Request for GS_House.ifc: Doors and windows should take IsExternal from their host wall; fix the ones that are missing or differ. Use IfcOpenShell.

First a look at what the model holds.

```python
import ifcopenshell
import ifcopenshell.util.element

model = ifcopenshell.open("GS_House.ifc")
print(model.schema)
seen = {}
for e in model.by_type("IfcDoor") + model.by_type("IfcWindow"):
    if not e.FillsVoids:
        continue
    host = e.FillsVoids[0].RelatingOpeningElement.VoidsElements[0].RelatingBuildingElement
    own = ifcopenshell.util.element.get_pset(e, f"Pset_{e.is_a()[3:].removesuffix('StandardCase')}Common", "IsExternal")
    wall = ifcopenshell.util.element.get_pset(host, "Pset_WallCommon", "IsExternal")
    seen[e.is_a(), own, wall] = seen.get((e.is_a(), own, wall), 0) + 1
for (cls, own, wall), count in sorted(seen.items(), key=str):
    print(count, cls, "IsExternal:", own, "| host wall:", wall)
```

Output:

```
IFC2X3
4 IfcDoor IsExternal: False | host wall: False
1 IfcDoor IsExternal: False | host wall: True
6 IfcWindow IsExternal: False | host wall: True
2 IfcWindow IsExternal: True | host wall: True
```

```python
import ifcopenshell
import ifcopenshell.api.pset
import ifcopenshell.util.element

model = ifcopenshell.open("GS_House.ifc")

count = 0
for ifc_class, pset_name in (("IfcDoor", "Pset_DoorCommon"), ("IfcWindow", "Pset_WindowCommon")):
    for e in model.by_type(ifc_class):
        if not e.FillsVoids:
            continue
        host = e.FillsVoids[0].RelatingOpeningElement.VoidsElements[0].RelatingBuildingElement
        external = ifcopenshell.util.element.get_pset(host, "Pset_WallCommon", "IsExternal")
        if external is None or ifcopenshell.util.element.get_pset(e, pset_name, "IsExternal") == external:
            continue
        pset = ifcopenshell.api.pset.add_pset(model, product=e, name=pset_name)
        ifcopenshell.api.pset.edit_pset(model, pset=pset, properties={"IsExternal": external})
        count += 1

print(count, "updated")

model.write("GS_House_edited.ifc")
```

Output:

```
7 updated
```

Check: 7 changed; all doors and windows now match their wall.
